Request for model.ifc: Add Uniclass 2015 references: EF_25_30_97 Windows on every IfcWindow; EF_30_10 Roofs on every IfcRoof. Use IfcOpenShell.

First a look at what the model holds.

```python
import ifcopenshell

model = ifcopenshell.open("model.ifc")
print(model.schema)
print("classifications:", [c.Name for c in model.by_type("IfcClassification")])
for ifc_class in ("IfcDoor", "IfcRoof", "IfcStair", "IfcWall", "IfcWindow"):
    print(ifc_class, len(model.by_type(ifc_class)))
```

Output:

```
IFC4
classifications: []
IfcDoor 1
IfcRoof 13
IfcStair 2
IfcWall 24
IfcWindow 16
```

```python
import ifcopenshell
import ifcopenshell.api.classification

model = ifcopenshell.open("model.ifc")

system = ifcopenshell.api.classification.add_classification(model, classification="Uniclass 2015")

codes = {
    "IfcWindow": ("EF_25_30_97", "Windows"),
    "IfcRoof": ("EF_30_10", "Roofs"),
}
for ifc_class, (code, name) in codes.items():
    products = model.by_type(ifc_class)
    ifcopenshell.api.classification.add_reference(
        model, products=products, classification=system, identification=code, name=name
    )
    print(code, len(products))

model.write("model_edited.ifc")
```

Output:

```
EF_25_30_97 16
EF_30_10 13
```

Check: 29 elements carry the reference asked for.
